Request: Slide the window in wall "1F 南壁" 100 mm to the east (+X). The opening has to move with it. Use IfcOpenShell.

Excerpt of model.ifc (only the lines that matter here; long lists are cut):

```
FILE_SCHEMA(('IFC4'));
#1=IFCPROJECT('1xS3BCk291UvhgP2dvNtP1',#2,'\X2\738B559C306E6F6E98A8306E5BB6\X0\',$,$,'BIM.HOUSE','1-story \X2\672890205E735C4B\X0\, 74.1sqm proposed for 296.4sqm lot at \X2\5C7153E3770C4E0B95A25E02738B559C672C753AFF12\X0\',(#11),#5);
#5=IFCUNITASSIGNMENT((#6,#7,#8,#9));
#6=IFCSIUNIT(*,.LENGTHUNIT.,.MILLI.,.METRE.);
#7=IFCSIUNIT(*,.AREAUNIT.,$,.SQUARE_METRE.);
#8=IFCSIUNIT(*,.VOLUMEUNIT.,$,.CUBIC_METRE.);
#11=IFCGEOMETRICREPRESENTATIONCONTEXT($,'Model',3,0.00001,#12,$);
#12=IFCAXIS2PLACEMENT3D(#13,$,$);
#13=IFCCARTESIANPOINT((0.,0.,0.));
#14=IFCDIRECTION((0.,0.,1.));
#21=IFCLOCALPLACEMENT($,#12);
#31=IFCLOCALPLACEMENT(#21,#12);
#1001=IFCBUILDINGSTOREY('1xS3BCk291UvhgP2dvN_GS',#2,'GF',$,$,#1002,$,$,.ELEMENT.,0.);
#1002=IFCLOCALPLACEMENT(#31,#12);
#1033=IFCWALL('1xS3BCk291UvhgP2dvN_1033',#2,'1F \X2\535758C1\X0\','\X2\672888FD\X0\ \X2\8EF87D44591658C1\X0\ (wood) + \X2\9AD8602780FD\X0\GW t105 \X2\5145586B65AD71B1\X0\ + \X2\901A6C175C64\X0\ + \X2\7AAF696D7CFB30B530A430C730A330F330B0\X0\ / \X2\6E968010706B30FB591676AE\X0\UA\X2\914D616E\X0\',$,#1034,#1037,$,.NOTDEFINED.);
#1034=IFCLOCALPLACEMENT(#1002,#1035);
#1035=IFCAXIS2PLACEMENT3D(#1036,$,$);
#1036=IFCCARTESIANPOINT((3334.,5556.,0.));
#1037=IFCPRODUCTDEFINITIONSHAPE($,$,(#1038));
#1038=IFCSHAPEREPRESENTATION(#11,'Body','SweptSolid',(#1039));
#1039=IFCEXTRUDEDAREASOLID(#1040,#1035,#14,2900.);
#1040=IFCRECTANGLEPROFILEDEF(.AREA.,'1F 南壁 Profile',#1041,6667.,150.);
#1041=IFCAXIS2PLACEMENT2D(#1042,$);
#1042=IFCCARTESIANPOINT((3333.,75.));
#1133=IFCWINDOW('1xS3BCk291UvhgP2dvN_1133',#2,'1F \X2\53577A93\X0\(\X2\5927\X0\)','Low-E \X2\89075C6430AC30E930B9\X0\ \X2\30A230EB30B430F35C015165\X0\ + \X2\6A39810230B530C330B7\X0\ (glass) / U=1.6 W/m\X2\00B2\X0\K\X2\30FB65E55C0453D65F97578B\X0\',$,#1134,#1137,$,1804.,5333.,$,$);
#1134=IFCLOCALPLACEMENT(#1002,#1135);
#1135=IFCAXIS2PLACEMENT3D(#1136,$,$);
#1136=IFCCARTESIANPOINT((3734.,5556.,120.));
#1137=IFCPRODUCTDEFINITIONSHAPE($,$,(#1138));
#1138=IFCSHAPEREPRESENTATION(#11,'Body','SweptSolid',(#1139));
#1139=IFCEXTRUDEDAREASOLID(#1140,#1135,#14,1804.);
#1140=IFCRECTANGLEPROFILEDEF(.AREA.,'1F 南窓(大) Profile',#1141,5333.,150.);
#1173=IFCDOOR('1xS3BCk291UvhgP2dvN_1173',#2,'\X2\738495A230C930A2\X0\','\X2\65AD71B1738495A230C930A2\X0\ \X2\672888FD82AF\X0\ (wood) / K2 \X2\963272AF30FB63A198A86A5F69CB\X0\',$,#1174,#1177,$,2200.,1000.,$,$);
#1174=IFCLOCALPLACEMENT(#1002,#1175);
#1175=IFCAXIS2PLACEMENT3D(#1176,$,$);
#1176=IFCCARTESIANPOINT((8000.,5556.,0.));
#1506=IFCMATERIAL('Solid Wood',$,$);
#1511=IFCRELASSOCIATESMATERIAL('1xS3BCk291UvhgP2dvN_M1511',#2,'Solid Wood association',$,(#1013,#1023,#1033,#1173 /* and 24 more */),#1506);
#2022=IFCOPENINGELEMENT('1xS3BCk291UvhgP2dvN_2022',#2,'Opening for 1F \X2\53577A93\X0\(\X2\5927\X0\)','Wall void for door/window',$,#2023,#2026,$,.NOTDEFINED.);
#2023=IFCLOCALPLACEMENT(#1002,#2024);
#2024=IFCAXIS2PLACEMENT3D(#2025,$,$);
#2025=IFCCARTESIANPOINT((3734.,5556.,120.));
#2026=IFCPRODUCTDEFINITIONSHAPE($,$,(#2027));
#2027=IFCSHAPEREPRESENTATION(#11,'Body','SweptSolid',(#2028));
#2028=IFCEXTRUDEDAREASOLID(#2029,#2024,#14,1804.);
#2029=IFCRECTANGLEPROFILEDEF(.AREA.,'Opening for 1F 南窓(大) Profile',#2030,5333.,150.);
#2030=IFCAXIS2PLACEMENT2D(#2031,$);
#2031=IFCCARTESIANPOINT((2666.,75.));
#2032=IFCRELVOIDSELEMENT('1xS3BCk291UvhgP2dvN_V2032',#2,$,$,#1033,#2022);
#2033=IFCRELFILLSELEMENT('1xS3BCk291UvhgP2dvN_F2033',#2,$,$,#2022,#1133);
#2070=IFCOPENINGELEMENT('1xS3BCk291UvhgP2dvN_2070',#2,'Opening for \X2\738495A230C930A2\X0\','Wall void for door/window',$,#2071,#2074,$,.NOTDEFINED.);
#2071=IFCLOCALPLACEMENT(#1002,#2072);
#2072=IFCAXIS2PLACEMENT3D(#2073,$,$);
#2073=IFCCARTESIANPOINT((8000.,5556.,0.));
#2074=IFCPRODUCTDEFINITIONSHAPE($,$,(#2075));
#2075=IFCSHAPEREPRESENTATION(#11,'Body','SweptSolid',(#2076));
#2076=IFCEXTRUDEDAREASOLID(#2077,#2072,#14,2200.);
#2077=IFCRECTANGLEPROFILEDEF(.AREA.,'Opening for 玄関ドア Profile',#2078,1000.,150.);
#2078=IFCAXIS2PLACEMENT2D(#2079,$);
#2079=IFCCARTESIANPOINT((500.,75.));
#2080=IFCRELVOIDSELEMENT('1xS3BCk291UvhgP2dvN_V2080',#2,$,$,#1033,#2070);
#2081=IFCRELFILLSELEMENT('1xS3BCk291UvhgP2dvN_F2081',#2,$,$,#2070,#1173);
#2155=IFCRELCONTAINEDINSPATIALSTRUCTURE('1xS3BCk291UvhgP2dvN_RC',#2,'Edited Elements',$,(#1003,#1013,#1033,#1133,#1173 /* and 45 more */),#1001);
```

```python
import ifcopenshell
import ifcopenshell.api.geometry
import ifcopenshell.util.placement

model = ifcopenshell.open("model.ifc")

window = model.by_guid("1xS3BCk291UvhgP2dvN_1133")
opening = window.FillsVoids[0].RelatingOpeningElement
wall = opening.VoidsElements[0].RelatingBuildingElement

wall_matrix = ifcopenshell.util.placement.get_local_placement(wall.ObjectPlacement)
shift = wall_matrix[:3, 0] * 100.0
before = ifcopenshell.util.placement.get_local_placement(window.ObjectPlacement)[:3, 3].copy()

# The window is not placed relative to its opening, so move both.
for product in (opening, window):
    matrix = ifcopenshell.util.placement.get_local_placement(product.ObjectPlacement)
    matrix[:3, 3] += shift
    ifcopenshell.api.geometry.edit_object_placement(model, product=product, matrix=matrix, is_si=False)

after = ifcopenshell.util.placement.get_local_placement(window.ObjectPlacement)[:3, 3]
print("window moved by", (after - before).round(3) + 0.0)

model.write("model_updated.ifc")
```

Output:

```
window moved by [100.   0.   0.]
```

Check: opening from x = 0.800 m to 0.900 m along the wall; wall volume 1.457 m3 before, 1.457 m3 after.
